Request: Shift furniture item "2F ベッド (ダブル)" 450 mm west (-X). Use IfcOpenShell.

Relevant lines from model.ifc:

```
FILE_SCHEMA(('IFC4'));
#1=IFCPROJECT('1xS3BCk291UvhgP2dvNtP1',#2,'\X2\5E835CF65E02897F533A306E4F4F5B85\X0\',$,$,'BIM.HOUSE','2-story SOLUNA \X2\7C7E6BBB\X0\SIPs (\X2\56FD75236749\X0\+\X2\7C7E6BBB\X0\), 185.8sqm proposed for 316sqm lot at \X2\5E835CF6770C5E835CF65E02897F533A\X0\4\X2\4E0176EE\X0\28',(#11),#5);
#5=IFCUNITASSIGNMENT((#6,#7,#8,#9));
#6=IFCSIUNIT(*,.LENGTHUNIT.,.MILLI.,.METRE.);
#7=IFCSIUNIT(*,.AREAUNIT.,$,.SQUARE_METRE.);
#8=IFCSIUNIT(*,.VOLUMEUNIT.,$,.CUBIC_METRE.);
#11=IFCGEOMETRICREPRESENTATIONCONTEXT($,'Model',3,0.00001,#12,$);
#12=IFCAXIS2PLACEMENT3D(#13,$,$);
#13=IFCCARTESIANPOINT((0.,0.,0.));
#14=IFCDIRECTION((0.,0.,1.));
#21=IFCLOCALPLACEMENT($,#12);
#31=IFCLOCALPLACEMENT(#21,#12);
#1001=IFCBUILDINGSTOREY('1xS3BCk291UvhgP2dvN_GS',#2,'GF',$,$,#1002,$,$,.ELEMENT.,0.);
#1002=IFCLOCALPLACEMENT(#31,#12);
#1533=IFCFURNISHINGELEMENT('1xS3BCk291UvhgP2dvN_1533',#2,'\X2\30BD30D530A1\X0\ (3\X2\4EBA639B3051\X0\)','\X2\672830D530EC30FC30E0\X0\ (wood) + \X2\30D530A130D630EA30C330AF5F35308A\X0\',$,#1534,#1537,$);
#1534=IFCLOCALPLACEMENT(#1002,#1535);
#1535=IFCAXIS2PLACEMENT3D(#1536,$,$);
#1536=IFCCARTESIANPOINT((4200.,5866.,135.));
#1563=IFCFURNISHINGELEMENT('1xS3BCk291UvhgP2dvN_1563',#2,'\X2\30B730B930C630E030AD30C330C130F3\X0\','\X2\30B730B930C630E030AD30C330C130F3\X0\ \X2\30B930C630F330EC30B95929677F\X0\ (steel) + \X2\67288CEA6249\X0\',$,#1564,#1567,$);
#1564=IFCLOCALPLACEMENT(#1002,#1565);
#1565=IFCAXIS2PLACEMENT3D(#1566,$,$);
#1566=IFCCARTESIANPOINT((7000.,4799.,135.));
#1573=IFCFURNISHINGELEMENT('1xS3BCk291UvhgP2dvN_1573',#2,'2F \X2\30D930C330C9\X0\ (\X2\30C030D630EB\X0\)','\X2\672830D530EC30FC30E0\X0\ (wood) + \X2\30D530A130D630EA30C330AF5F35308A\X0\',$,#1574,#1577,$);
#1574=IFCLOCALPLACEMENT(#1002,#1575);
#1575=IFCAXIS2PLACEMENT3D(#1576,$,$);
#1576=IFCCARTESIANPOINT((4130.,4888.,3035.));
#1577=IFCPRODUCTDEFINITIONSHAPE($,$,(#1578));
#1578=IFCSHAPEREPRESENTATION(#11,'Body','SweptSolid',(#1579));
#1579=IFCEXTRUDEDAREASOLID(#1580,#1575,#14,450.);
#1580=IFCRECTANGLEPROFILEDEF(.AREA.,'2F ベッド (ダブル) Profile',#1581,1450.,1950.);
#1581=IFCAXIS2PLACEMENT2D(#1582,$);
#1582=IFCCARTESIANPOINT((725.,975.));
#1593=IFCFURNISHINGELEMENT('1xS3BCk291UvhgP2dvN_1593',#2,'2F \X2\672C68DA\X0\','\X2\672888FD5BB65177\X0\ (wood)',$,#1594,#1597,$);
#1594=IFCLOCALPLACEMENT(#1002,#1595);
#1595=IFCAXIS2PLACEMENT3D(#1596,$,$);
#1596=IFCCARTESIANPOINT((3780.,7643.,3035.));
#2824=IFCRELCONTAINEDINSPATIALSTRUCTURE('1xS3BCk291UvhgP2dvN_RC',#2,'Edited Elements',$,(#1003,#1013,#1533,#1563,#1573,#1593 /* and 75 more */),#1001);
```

```python
import ifcopenshell
import ifcopenshell.api.geometry
import ifcopenshell.util.placement

model = ifcopenshell.open("model.ifc")

item = model.by_guid("1xS3BCk291UvhgP2dvN_1573")
matrix = ifcopenshell.util.placement.get_local_placement(item.ObjectPlacement)
matrix[0, 3] -= 450.0
ifcopenshell.api.geometry.edit_object_placement(model, product=item, matrix=matrix, is_si=False)

print(ifcopenshell.util.placement.get_local_placement(item.ObjectPlacement).round(3) + 0.0)

model.write("model-out.ifc")
```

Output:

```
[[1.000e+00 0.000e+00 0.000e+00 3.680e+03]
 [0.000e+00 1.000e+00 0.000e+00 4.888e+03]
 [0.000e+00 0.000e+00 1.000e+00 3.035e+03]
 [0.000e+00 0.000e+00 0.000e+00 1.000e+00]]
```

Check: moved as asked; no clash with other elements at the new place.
